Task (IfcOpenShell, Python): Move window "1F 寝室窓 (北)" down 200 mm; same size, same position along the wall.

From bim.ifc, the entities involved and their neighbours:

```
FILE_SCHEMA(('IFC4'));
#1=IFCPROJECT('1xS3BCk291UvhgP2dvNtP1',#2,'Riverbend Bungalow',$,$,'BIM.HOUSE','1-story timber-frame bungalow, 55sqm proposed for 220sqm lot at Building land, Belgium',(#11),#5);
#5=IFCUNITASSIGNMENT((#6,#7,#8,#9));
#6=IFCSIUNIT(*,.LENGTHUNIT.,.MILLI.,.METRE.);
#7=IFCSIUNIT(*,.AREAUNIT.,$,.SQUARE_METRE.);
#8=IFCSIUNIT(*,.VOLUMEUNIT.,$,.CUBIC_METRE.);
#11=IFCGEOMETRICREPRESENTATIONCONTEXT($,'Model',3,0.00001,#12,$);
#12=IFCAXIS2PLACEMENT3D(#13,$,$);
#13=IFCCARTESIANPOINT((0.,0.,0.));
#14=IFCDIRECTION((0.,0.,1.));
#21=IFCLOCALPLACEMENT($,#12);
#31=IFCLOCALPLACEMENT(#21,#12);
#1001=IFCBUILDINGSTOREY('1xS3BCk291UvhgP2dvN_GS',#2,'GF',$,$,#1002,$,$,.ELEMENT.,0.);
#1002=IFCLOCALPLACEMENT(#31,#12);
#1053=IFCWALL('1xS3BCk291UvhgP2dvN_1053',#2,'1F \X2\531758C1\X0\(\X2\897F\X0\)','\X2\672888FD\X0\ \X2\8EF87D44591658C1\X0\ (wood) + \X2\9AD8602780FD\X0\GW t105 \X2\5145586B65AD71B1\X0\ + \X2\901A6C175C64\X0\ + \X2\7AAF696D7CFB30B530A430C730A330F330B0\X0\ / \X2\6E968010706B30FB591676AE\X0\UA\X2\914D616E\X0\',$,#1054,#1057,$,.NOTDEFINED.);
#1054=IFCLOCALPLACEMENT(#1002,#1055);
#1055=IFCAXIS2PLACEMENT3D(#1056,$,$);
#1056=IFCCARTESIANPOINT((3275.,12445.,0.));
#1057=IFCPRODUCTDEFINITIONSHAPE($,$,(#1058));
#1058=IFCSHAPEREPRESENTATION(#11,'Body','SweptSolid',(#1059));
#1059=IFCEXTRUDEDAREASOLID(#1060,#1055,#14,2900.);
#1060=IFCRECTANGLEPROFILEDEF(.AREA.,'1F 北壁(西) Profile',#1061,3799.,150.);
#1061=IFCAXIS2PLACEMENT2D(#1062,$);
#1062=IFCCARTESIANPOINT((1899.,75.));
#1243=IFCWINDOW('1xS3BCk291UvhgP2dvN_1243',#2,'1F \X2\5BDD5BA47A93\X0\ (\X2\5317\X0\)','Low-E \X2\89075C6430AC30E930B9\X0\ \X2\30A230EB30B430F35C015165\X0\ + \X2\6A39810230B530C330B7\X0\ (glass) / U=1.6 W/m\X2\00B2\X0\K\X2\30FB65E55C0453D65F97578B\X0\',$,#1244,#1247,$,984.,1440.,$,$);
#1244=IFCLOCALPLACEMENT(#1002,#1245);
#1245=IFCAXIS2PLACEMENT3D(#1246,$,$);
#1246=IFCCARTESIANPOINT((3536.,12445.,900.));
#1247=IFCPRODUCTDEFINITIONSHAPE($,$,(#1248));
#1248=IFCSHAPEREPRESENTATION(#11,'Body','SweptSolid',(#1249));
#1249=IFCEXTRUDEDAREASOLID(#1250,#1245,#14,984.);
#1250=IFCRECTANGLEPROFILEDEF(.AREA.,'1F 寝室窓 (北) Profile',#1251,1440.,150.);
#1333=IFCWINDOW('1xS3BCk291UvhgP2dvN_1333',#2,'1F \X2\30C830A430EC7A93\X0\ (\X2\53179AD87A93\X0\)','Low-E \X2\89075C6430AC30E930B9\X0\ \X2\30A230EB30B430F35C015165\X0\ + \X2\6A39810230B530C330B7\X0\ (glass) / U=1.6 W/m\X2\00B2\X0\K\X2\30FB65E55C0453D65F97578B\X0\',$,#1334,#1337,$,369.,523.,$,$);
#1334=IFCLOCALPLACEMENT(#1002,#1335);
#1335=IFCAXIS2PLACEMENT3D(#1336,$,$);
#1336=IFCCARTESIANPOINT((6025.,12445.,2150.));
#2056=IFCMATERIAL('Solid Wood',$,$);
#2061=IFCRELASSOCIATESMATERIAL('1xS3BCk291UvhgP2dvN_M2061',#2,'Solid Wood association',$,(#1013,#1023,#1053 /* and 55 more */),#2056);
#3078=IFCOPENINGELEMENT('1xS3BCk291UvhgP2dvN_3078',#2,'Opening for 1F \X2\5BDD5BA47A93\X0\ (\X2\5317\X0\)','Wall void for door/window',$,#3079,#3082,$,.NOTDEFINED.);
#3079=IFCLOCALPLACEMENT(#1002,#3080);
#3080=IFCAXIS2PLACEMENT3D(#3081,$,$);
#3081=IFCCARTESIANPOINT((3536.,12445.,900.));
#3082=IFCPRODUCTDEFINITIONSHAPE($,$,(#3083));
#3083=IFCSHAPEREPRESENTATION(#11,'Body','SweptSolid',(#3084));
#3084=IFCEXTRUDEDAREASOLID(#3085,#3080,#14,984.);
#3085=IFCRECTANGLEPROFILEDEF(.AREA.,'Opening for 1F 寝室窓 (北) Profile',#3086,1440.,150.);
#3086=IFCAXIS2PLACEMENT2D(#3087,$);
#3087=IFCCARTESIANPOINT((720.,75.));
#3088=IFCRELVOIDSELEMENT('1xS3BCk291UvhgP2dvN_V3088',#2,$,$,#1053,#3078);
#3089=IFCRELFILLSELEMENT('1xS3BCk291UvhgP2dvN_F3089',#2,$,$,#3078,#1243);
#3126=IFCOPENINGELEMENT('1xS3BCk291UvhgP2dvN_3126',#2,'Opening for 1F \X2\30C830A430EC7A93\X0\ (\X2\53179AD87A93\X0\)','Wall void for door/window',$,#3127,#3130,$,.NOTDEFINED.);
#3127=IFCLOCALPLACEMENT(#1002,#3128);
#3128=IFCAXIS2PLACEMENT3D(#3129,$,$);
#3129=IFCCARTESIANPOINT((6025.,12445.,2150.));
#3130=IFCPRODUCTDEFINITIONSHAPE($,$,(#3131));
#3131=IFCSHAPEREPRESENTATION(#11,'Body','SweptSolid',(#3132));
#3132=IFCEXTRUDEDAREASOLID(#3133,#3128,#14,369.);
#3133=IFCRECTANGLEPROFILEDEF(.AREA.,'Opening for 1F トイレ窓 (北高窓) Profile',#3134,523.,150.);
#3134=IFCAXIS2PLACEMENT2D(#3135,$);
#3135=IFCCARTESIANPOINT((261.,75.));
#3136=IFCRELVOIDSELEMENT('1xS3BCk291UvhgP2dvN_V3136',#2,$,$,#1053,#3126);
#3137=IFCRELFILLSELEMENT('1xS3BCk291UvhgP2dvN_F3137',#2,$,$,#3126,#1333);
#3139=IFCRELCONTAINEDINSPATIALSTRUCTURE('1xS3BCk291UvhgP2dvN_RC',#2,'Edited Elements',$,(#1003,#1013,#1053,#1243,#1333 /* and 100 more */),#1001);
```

```python
import numpy as np
import ifcopenshell
import ifcopenshell.api.geometry
import ifcopenshell.util.placement
import ifcopenshell.util.unit

model = ifcopenshell.open("bim.ifc")
unit_scale = ifcopenshell.util.unit.calculate_unit_scale(model)

window = model.by_id(1243)
opening = window.FillsVoids[0].RelatingOpeningElement
dz = -0.2 / unit_scale

shift = np.array([0.0, 0.0, dz])
# The window is not placed relative to its opening, so move both.
for product in (opening, window):
    matrix = ifcopenshell.util.placement.get_local_placement(product.ObjectPlacement)
    matrix[:3, 3] += shift
    ifcopenshell.api.geometry.edit_object_placement(model, product=product, matrix=matrix, is_si=False)

print(f"moved by {dz * unit_scale:+.3f} m")

model.write("bim_edited.ifc")
```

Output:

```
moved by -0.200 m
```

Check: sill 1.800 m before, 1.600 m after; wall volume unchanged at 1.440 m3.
